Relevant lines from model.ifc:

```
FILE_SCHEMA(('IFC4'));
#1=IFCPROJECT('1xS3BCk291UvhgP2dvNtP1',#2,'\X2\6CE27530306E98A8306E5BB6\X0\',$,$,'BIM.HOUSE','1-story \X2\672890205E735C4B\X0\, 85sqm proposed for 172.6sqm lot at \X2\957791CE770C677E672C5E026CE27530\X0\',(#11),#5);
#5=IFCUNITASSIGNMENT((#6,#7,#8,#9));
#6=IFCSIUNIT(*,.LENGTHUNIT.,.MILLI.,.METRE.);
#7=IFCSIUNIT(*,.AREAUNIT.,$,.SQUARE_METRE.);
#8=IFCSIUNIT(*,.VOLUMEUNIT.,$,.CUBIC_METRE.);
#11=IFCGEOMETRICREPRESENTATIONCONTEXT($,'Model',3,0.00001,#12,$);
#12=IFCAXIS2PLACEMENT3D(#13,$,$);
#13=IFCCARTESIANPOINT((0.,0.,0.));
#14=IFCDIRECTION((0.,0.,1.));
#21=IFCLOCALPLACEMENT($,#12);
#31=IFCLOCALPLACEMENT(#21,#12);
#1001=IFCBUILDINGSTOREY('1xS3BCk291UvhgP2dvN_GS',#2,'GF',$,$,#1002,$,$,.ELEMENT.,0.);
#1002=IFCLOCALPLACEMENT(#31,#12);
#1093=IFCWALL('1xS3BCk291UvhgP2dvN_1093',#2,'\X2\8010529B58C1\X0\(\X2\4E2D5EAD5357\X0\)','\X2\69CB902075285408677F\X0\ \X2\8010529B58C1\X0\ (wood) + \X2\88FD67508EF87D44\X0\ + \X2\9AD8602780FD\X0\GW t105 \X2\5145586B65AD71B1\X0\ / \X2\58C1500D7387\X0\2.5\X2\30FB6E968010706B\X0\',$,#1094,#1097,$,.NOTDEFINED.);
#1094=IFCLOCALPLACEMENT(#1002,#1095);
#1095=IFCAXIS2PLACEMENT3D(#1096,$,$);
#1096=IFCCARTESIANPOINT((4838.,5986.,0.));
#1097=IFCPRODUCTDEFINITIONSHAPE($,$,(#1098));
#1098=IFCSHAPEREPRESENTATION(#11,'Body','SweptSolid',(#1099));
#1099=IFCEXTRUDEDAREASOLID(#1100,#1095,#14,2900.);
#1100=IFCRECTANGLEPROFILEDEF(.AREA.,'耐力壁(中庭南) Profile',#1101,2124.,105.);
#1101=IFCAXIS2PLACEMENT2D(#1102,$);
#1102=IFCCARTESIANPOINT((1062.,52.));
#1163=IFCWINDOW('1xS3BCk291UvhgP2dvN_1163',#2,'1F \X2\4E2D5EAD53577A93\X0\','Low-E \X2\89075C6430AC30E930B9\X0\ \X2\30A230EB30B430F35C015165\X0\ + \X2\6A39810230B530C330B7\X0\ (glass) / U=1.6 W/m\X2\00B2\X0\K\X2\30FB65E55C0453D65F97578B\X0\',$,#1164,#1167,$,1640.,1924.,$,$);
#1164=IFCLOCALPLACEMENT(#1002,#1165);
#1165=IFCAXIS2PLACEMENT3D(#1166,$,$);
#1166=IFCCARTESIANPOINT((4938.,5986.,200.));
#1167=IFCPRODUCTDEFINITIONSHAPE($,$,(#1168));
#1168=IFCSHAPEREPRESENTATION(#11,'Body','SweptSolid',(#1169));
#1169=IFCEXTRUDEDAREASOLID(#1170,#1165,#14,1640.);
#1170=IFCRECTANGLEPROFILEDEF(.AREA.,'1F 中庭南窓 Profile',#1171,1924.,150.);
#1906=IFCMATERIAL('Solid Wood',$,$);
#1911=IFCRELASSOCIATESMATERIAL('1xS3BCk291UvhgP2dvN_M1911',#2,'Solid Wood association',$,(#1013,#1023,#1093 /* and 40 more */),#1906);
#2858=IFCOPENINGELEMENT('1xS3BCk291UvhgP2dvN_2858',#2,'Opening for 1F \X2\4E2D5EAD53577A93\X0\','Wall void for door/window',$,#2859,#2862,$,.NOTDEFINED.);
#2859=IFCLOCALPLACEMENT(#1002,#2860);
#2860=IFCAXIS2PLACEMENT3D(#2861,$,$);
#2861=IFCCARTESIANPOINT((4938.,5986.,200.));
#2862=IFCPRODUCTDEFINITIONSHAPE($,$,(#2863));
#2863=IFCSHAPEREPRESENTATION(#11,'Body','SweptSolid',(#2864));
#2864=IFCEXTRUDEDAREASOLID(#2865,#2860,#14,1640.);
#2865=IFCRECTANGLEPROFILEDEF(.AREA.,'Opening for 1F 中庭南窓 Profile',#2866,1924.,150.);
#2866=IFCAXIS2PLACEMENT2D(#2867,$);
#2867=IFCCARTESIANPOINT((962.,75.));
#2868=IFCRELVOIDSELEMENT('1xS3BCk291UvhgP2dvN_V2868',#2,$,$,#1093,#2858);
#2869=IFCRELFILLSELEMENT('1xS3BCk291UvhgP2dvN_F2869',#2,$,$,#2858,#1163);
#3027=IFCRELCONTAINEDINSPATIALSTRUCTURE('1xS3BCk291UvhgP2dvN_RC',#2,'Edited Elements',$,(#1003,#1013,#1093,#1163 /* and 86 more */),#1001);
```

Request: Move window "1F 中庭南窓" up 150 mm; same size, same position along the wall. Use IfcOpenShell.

```python
import numpy as np
import ifcopenshell
import ifcopenshell.api.geometry
import ifcopenshell.util.placement
import ifcopenshell.util.unit

model = ifcopenshell.open("model.ifc")
unit_scale = ifcopenshell.util.unit.calculate_unit_scale(model)

window = model.by_id(1163)
opening = window.FillsVoids[0].RelatingOpeningElement
dz = 150.0

shift = np.array([0.0, 0.0, dz])
# The window is not placed relative to its opening, so move both.
for product in (opening, window):
    matrix = ifcopenshell.util.placement.get_local_placement(product.ObjectPlacement)
    matrix[:3, 3] += shift
    ifcopenshell.api.geometry.edit_object_placement(model, product=product, matrix=matrix, is_si=False)

print(f"moved by {dz * unit_scale:+.3f} m")

model.write("model_v2.ifc")
```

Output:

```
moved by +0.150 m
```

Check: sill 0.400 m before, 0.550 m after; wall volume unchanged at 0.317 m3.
